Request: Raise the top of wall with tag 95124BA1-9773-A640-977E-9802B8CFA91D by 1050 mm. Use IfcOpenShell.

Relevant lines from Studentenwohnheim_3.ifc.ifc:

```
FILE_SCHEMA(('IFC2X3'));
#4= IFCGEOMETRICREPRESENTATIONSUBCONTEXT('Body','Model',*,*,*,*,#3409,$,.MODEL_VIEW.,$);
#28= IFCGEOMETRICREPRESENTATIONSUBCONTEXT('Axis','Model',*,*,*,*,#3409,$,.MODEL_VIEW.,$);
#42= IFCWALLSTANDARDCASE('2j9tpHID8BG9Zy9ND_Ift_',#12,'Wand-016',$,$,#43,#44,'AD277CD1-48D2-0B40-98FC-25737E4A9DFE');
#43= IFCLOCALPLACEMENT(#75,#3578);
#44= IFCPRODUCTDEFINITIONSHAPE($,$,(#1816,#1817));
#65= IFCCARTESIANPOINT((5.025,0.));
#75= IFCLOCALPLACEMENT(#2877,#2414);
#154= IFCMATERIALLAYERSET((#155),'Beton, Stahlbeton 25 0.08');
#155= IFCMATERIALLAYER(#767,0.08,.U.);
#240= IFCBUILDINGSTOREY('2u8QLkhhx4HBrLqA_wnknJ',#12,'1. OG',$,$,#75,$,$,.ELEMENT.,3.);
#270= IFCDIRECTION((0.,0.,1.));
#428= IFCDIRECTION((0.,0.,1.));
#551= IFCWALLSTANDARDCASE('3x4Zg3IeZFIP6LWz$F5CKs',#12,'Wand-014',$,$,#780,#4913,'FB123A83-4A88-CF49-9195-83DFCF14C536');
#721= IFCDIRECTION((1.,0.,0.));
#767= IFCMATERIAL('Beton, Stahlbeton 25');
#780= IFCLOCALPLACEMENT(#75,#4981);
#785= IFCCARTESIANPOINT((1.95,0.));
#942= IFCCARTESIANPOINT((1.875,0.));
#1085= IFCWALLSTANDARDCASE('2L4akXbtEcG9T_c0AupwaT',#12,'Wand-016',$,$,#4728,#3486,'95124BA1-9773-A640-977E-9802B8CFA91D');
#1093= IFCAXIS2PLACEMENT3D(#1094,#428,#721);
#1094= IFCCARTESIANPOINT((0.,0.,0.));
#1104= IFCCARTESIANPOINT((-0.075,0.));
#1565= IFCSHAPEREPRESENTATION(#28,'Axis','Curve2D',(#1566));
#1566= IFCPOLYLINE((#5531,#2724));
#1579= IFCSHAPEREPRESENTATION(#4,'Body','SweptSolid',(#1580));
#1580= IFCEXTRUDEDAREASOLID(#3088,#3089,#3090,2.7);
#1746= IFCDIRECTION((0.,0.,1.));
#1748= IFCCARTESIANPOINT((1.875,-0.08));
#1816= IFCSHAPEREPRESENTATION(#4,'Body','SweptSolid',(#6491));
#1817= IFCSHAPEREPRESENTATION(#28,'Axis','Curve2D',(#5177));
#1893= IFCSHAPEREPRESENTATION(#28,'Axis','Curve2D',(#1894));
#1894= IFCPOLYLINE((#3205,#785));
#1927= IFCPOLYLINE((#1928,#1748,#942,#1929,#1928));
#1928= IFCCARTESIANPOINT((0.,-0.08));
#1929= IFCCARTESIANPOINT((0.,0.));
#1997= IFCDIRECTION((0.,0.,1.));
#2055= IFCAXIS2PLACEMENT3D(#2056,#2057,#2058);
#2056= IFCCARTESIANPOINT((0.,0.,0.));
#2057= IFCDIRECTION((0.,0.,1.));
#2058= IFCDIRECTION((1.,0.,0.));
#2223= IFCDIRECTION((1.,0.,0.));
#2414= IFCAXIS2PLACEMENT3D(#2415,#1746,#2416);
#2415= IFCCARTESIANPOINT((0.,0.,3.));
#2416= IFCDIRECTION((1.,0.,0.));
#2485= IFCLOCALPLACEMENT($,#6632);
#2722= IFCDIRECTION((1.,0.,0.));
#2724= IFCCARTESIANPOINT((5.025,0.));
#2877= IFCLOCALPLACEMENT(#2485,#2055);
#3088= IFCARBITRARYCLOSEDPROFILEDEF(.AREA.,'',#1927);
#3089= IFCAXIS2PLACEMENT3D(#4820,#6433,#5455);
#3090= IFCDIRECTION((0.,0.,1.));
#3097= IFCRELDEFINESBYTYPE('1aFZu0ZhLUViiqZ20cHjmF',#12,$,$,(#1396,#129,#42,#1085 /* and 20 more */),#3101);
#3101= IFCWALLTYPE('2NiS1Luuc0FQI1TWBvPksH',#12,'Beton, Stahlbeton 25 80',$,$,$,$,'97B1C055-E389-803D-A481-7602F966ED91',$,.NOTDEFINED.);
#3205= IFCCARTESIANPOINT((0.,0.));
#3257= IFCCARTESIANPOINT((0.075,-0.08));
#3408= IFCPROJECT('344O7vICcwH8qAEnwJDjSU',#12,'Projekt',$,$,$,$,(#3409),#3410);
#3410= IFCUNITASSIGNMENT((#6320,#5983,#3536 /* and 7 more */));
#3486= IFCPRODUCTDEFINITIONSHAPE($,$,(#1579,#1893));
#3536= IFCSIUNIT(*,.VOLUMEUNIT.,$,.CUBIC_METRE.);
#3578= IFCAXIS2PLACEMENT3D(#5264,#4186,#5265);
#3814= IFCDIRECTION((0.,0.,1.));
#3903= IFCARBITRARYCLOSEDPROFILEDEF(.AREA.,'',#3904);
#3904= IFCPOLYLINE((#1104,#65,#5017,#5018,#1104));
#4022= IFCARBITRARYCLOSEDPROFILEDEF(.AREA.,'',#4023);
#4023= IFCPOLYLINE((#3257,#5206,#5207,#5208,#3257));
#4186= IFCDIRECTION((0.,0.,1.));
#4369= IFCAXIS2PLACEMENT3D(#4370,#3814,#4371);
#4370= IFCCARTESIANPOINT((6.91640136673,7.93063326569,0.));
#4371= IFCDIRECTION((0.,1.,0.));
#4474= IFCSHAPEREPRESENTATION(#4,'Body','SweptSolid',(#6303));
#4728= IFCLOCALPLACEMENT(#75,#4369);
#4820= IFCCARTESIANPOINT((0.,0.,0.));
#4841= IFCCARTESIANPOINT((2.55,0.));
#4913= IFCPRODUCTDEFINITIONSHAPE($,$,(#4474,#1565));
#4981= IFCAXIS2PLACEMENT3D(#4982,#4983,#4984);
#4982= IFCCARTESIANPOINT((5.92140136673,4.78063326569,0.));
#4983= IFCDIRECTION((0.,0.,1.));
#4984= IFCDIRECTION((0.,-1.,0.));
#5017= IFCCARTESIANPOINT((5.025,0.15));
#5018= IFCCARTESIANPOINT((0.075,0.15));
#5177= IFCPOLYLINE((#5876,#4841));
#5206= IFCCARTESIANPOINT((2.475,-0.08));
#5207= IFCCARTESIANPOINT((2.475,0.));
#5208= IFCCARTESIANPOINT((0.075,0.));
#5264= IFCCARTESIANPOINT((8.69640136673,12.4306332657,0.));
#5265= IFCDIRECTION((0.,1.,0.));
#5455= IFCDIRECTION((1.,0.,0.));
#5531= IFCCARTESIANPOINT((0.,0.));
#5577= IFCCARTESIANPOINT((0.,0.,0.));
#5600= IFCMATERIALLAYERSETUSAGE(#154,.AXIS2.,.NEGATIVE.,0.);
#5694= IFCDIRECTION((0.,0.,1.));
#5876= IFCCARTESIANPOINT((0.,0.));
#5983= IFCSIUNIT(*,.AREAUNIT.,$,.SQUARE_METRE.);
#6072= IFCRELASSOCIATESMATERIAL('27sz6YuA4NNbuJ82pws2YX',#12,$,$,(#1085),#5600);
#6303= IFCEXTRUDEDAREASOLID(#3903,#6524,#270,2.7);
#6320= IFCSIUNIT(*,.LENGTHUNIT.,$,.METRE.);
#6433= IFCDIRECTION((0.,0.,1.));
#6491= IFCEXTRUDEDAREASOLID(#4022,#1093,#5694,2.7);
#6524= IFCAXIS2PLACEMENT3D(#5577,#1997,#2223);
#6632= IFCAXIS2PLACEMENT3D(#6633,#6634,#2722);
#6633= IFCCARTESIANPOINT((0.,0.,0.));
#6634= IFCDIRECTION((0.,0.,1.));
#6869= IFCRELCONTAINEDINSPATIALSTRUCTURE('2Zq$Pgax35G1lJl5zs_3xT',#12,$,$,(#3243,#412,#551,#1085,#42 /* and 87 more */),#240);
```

```python
import ifcopenshell
import ifcopenshell.geom
import ifcopenshell.util.representation
import ifcopenshell.util.shape
import ifcopenshell.util.unit

model = ifcopenshell.open("Studentenwohnheim_3.ifc.ifc")
unit_scale = ifcopenshell.util.unit.calculate_unit_scale(model)
settings = ifcopenshell.geom.settings()


def volume(element):
    """Net volume in cubic metres, openings subtracted."""
    shape = ifcopenshell.geom.create_shape(settings, element)
    return ifcopenshell.util.shape.get_volume(shape.geometry)


wall = model.by_guid("2L4akXbtEcG9T_c0AupwaT")
before = volume(wall)

body = ifcopenshell.util.representation.get_representation(wall, "Model", "Body")
solid = body.Items[0]
old_height = solid.Depth
solid.Depth += 1.05 / unit_scale
after = volume(wall)

print(f"height {old_height:g} -> {solid.Depth:g}, volume {before:.3f} -> {after:.3f} m3")

model.write("Studentenwohnheim_3.ifc_updated.ifc")
```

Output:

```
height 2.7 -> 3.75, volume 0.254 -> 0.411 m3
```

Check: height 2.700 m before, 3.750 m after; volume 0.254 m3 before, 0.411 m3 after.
